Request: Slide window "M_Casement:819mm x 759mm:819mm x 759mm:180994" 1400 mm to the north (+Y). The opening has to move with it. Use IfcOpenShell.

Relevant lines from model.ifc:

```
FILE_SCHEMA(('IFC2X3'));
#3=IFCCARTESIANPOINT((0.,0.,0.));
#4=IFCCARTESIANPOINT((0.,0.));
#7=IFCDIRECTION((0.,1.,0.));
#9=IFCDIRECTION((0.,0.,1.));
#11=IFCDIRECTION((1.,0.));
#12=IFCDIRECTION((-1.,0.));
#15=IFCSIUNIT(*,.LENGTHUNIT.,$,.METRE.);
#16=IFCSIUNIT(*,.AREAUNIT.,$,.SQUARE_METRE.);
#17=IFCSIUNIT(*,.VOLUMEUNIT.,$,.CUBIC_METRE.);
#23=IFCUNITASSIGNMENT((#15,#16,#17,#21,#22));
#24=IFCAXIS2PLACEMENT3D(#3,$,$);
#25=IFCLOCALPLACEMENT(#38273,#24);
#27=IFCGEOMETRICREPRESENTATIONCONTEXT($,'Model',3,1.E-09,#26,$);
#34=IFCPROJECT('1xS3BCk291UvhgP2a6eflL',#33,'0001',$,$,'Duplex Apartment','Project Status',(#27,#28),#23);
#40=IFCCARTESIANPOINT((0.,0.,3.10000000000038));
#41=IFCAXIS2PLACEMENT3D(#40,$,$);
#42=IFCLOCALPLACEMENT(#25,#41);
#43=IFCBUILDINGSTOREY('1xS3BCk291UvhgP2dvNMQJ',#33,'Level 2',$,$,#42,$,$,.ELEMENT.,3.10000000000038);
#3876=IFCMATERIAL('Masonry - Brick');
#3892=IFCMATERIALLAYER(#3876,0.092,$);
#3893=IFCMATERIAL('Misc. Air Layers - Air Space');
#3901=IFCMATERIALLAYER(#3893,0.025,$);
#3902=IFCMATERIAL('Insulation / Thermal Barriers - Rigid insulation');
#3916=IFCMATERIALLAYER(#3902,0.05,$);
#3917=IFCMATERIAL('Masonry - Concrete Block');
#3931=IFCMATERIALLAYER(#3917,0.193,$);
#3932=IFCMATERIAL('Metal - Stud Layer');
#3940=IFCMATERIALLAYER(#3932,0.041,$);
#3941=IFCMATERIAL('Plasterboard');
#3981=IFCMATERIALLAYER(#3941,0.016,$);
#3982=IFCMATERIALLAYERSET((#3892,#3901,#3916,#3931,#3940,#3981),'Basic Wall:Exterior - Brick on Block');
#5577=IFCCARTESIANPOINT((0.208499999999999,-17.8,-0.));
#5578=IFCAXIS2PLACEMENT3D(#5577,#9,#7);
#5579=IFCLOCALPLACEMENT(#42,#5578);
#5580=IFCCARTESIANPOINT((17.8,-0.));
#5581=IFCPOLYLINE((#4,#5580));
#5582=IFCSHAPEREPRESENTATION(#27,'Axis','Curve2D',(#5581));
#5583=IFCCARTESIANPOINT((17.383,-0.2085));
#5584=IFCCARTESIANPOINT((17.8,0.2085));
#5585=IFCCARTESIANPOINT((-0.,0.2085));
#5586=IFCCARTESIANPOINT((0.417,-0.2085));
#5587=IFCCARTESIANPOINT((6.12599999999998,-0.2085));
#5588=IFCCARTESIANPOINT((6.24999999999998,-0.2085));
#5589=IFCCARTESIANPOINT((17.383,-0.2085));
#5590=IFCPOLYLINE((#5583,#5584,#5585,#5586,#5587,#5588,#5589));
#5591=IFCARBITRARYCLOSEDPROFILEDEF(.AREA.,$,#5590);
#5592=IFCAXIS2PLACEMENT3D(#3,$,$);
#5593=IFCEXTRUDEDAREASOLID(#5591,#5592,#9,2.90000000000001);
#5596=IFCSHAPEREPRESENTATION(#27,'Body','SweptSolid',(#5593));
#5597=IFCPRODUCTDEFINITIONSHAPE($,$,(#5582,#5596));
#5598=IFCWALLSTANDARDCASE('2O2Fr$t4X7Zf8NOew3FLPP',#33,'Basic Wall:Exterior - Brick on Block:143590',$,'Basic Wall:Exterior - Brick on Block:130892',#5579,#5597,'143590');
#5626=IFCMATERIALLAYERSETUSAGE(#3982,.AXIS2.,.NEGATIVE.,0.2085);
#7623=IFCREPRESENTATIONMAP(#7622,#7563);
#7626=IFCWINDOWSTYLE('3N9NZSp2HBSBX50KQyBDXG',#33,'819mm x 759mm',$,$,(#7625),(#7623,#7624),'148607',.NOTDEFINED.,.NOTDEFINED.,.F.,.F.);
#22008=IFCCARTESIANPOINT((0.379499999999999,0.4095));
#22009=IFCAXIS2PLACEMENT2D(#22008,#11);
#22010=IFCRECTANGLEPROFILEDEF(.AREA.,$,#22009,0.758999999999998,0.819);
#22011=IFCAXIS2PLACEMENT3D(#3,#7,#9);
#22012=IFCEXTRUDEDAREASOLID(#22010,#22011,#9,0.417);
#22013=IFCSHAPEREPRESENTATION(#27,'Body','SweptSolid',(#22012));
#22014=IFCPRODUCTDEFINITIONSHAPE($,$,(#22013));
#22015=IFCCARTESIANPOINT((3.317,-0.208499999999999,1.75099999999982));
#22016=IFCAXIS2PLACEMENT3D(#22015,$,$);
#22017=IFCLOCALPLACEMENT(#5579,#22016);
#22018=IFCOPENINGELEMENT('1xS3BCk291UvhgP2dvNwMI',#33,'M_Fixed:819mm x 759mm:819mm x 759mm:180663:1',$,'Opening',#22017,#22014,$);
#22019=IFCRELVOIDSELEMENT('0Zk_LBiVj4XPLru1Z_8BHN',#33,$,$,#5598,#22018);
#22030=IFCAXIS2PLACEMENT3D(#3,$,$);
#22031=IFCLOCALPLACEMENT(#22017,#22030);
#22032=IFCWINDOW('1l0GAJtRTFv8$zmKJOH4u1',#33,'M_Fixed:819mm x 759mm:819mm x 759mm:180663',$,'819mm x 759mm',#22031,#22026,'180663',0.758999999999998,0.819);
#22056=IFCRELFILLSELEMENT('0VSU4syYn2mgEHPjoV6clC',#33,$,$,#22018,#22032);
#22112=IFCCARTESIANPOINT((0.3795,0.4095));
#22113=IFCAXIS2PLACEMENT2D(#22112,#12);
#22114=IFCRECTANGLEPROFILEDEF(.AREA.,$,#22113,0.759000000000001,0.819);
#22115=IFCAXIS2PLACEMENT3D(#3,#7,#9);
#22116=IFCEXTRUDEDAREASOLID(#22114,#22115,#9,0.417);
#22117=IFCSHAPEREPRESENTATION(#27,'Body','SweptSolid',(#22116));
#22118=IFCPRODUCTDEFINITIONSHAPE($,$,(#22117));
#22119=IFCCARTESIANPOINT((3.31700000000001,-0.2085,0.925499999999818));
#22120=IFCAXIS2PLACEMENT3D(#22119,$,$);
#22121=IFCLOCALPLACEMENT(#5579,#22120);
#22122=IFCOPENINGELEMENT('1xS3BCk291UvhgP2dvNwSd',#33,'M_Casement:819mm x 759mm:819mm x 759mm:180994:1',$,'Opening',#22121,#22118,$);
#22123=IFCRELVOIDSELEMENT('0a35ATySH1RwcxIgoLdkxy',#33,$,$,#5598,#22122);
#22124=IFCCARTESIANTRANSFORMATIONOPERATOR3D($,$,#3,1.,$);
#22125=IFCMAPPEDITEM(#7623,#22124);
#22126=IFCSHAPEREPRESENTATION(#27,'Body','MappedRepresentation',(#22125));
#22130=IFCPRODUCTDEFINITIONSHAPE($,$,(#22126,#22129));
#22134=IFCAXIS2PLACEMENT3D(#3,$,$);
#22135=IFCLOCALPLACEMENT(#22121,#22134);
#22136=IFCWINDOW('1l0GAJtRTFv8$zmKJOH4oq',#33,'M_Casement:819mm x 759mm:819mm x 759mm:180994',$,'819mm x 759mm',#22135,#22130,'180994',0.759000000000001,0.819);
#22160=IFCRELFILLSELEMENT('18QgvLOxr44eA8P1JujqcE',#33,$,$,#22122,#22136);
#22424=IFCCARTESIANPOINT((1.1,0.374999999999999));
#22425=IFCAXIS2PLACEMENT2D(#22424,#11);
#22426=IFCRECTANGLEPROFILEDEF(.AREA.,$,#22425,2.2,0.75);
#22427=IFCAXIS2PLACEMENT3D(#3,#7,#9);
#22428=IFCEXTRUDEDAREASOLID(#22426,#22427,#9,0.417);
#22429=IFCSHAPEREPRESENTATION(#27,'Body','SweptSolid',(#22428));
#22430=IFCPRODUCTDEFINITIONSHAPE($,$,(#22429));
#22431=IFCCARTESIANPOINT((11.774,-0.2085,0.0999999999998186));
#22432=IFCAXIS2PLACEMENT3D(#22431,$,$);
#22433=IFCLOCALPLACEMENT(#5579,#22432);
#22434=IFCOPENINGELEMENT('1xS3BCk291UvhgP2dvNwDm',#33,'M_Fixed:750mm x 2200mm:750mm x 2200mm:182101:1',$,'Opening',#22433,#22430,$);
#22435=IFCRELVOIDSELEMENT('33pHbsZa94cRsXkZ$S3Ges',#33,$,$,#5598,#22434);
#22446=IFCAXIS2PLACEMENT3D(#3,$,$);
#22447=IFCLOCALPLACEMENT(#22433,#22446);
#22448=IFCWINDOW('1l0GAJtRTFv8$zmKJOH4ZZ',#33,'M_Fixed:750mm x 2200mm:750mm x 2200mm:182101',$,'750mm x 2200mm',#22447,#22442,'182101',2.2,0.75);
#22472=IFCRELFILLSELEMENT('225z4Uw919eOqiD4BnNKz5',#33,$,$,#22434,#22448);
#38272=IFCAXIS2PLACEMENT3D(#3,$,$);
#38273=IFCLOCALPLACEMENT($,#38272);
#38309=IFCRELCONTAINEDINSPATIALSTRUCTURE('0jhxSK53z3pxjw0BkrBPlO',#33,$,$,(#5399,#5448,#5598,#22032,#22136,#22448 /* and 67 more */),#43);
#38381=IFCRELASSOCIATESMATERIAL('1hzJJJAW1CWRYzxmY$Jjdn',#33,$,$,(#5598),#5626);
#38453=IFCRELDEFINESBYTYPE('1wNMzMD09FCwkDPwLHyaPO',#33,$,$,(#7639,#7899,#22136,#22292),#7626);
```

```python
import ifcopenshell
import ifcopenshell.api.geometry
import ifcopenshell.util.placement
import ifcopenshell.util.unit

model = ifcopenshell.open("model.ifc")
unit_scale = ifcopenshell.util.unit.calculate_unit_scale(model)

window = model.by_guid("1l0GAJtRTFv8$zmKJOH4oq")
opening = window.FillsVoids[0].RelatingOpeningElement
wall = opening.VoidsElements[0].RelatingBuildingElement

wall_matrix = ifcopenshell.util.placement.get_local_placement(wall.ObjectPlacement)
shift = wall_matrix[:3, 0] * 1.4 / unit_scale
before = ifcopenshell.util.placement.get_local_placement(window.ObjectPlacement)[:3, 3].copy()

# The window is placed relative to its opening, so it follows when the opening moves.
matrix = ifcopenshell.util.placement.get_local_placement(opening.ObjectPlacement)
matrix[:3, 3] += shift
ifcopenshell.api.geometry.edit_object_placement(
    model, product=opening, matrix=matrix, is_si=False, should_transform_children=True
)

after = ifcopenshell.util.placement.get_local_placement(window.ObjectPlacement)[:3, 3]
print("window moved by", (after - before).round(3) + 0.0)

model.write("model_rev.ifc")
```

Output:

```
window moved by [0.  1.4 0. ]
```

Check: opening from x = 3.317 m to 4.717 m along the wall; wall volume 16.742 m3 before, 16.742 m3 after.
